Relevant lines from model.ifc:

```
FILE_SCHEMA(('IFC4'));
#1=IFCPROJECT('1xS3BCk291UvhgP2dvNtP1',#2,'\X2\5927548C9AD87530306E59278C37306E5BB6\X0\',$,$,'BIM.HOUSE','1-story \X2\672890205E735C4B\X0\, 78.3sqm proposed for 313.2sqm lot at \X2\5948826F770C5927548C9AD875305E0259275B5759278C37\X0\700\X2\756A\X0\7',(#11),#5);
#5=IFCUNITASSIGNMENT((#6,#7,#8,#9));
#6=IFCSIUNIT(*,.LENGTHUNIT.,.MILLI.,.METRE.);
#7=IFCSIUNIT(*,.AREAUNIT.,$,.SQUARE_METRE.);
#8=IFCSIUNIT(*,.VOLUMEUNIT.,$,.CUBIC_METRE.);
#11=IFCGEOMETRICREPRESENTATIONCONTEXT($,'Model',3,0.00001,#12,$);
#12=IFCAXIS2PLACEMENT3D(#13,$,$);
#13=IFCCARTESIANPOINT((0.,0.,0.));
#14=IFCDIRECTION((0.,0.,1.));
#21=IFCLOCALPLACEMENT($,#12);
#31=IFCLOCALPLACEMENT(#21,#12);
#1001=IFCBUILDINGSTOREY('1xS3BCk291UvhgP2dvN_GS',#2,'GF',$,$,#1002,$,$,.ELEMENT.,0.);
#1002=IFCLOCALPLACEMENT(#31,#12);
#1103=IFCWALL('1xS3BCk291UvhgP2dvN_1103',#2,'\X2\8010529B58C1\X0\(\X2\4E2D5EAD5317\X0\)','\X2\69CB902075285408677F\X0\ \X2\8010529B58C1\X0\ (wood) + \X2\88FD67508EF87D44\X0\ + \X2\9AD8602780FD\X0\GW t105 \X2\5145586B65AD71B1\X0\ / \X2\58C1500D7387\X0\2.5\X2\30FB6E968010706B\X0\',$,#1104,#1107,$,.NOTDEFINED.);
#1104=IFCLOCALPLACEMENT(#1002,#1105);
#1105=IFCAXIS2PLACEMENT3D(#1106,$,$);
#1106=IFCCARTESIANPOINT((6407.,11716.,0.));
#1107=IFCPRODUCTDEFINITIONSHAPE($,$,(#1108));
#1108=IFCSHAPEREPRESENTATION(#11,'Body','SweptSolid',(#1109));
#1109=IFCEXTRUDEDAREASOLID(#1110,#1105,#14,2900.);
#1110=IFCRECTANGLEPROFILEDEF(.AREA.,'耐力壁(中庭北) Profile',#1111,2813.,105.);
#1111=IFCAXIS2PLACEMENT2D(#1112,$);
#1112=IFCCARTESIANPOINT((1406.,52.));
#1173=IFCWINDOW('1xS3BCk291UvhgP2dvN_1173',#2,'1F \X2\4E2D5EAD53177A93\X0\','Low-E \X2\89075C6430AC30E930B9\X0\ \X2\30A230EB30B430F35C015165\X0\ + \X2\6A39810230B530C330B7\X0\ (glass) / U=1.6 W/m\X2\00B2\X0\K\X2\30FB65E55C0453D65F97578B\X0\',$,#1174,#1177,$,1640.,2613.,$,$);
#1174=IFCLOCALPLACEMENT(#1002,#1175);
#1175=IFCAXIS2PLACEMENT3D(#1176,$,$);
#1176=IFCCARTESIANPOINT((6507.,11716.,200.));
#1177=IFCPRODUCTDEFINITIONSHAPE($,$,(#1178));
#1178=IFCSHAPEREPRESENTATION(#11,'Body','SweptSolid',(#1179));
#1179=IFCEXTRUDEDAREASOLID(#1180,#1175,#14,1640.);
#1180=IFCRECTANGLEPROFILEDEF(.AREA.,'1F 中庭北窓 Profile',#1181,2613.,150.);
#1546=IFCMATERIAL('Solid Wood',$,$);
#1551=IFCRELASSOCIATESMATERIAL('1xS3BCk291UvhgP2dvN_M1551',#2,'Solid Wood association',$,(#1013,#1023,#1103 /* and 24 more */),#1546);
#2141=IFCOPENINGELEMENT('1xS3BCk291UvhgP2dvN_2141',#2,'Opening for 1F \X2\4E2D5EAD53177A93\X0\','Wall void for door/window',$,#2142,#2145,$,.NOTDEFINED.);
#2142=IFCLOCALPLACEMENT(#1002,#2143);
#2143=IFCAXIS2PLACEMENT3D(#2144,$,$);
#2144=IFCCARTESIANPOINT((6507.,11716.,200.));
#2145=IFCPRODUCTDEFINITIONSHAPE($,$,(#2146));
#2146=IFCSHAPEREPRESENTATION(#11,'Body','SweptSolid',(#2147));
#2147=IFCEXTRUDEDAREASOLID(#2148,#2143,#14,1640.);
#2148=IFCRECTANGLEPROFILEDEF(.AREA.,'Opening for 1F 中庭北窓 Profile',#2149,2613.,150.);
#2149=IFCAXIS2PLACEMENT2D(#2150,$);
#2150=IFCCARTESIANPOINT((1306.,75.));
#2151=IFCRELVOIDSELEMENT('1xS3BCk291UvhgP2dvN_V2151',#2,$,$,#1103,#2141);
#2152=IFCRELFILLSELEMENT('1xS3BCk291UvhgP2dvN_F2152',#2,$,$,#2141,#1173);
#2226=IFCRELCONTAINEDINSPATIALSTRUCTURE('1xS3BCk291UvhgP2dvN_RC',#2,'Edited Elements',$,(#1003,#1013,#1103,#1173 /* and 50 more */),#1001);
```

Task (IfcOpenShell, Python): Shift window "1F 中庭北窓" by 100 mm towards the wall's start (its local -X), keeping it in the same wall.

```python
import ifcopenshell
import ifcopenshell.api.geometry
import ifcopenshell.util.placement
import ifcopenshell.util.unit

model = ifcopenshell.open("model.ifc")
unit_scale = ifcopenshell.util.unit.calculate_unit_scale(model)

window = model.by_guid("1xS3BCk291UvhgP2dvN_1173")
opening = window.FillsVoids[0].RelatingOpeningElement
wall = opening.VoidsElements[0].RelatingBuildingElement

wall_matrix = ifcopenshell.util.placement.get_local_placement(wall.ObjectPlacement)
shift = wall_matrix[:3, 0] * -0.1 / unit_scale
before = ifcopenshell.util.placement.get_local_placement(window.ObjectPlacement)[:3, 3].copy()

# The window is not placed relative to its opening, so move both.
for product in (opening, window):
    matrix = ifcopenshell.util.placement.get_local_placement(product.ObjectPlacement)
    matrix[:3, 3] += shift
    ifcopenshell.api.geometry.edit_object_placement(model, product=product, matrix=matrix, is_si=False)

after = ifcopenshell.util.placement.get_local_placement(window.ObjectPlacement)[:3, 3]
print("window moved by", (after - before).round(3) + 0.0)

model.write("model_rev.ifc")
```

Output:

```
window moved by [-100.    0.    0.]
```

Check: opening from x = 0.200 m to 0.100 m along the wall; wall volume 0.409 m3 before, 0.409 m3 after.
